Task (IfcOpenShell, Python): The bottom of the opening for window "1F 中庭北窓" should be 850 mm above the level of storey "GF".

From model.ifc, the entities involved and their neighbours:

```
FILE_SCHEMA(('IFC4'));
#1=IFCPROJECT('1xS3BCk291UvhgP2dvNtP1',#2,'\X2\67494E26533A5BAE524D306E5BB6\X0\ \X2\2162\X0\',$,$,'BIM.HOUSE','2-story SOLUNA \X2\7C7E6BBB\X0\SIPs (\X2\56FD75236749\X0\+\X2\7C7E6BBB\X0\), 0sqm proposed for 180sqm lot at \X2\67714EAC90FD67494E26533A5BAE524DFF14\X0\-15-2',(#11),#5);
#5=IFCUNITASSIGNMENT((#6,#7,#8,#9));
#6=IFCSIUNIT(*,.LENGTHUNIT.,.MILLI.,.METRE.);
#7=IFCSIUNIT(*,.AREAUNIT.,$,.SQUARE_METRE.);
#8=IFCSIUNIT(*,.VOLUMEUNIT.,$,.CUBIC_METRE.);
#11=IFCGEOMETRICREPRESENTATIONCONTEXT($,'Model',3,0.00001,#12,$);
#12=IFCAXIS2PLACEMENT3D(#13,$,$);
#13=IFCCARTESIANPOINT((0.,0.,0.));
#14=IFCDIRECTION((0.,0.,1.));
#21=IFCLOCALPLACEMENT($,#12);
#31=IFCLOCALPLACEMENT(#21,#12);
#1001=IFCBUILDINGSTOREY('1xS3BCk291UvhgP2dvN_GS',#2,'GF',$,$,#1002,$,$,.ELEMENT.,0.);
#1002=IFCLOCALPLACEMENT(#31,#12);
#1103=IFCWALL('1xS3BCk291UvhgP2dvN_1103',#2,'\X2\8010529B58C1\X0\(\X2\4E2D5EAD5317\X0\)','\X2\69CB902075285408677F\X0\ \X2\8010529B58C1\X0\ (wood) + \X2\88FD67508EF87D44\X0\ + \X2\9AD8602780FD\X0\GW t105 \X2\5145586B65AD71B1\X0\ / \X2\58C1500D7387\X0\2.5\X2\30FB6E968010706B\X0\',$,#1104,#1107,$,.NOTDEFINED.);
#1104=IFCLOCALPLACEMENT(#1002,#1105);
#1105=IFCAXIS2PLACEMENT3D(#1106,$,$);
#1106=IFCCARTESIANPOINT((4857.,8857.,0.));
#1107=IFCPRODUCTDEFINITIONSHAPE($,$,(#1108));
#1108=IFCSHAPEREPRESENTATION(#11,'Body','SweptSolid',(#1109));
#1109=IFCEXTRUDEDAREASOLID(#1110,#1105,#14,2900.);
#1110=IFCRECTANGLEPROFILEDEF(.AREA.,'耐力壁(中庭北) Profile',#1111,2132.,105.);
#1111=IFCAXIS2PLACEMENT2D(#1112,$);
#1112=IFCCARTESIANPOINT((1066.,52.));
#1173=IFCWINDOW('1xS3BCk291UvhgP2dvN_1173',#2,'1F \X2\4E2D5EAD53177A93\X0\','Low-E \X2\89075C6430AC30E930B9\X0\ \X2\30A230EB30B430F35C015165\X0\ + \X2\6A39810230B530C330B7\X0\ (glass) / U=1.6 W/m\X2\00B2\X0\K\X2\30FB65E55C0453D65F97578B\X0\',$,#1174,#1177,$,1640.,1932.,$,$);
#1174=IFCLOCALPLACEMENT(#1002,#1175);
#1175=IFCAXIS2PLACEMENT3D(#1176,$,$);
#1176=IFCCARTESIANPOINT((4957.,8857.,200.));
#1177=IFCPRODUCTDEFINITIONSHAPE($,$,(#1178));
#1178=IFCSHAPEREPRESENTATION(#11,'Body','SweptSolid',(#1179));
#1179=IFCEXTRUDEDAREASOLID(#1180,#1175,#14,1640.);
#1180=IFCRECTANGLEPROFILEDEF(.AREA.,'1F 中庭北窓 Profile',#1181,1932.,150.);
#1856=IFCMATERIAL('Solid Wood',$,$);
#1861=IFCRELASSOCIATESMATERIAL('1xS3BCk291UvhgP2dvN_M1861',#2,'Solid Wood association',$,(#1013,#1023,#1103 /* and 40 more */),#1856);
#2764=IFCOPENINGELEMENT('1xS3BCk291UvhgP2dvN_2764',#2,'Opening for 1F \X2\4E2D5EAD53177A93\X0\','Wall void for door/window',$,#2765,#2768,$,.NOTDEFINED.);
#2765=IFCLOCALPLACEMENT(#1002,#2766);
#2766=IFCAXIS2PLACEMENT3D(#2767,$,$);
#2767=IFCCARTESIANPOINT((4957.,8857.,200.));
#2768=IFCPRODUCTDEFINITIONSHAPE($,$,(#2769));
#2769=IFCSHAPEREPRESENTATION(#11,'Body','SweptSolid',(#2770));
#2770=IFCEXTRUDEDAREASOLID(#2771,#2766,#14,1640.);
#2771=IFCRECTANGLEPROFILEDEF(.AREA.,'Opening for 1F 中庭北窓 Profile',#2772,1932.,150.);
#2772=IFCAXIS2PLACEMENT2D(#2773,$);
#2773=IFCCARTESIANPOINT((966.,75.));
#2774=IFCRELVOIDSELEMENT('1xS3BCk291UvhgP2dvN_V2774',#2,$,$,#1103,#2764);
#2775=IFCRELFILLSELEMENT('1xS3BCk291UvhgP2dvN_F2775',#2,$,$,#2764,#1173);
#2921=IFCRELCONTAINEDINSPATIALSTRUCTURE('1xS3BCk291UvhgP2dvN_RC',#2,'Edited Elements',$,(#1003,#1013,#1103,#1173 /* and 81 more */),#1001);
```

```python
import numpy as np
import ifcopenshell
import ifcopenshell.api.geometry
import ifcopenshell.geom
import ifcopenshell.util.element
import ifcopenshell.util.placement
import ifcopenshell.util.shape
import ifcopenshell.util.unit

model = ifcopenshell.open("model.ifc")
unit_scale = ifcopenshell.util.unit.calculate_unit_scale(model)

window = model.by_guid("1xS3BCk291UvhgP2dvN_1173")
opening = window.FillsVoids[0].RelatingOpeningElement
storey = ifcopenshell.util.element.get_container(window, ifc_class="IfcBuildingStorey")
level = ifcopenshell.util.placement.get_local_placement(storey.ObjectPlacement)[2, 3]

# The opening's origin need not be at the sill, so measure its lowest point.
shape = ifcopenshell.geom.create_shape(ifcopenshell.geom.settings(), opening)
bottom = ifcopenshell.util.shape.get_shape_bottom_elevation(shape, shape.geometry) / unit_scale
dz = level + 0.85 / unit_scale - bottom

shift = np.array([0.0, 0.0, dz])
# The window is not placed relative to its opening, so move both.
for product in (opening, window):
    matrix = ifcopenshell.util.placement.get_local_placement(product.ObjectPlacement)
    matrix[:3, 3] += shift
    ifcopenshell.api.geometry.edit_object_placement(model, product=product, matrix=matrix, is_si=False)

print(f"moved by {dz * unit_scale:+.3f} m")

model.write("model-out.ifc")
```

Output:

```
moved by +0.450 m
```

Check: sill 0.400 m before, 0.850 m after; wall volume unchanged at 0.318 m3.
